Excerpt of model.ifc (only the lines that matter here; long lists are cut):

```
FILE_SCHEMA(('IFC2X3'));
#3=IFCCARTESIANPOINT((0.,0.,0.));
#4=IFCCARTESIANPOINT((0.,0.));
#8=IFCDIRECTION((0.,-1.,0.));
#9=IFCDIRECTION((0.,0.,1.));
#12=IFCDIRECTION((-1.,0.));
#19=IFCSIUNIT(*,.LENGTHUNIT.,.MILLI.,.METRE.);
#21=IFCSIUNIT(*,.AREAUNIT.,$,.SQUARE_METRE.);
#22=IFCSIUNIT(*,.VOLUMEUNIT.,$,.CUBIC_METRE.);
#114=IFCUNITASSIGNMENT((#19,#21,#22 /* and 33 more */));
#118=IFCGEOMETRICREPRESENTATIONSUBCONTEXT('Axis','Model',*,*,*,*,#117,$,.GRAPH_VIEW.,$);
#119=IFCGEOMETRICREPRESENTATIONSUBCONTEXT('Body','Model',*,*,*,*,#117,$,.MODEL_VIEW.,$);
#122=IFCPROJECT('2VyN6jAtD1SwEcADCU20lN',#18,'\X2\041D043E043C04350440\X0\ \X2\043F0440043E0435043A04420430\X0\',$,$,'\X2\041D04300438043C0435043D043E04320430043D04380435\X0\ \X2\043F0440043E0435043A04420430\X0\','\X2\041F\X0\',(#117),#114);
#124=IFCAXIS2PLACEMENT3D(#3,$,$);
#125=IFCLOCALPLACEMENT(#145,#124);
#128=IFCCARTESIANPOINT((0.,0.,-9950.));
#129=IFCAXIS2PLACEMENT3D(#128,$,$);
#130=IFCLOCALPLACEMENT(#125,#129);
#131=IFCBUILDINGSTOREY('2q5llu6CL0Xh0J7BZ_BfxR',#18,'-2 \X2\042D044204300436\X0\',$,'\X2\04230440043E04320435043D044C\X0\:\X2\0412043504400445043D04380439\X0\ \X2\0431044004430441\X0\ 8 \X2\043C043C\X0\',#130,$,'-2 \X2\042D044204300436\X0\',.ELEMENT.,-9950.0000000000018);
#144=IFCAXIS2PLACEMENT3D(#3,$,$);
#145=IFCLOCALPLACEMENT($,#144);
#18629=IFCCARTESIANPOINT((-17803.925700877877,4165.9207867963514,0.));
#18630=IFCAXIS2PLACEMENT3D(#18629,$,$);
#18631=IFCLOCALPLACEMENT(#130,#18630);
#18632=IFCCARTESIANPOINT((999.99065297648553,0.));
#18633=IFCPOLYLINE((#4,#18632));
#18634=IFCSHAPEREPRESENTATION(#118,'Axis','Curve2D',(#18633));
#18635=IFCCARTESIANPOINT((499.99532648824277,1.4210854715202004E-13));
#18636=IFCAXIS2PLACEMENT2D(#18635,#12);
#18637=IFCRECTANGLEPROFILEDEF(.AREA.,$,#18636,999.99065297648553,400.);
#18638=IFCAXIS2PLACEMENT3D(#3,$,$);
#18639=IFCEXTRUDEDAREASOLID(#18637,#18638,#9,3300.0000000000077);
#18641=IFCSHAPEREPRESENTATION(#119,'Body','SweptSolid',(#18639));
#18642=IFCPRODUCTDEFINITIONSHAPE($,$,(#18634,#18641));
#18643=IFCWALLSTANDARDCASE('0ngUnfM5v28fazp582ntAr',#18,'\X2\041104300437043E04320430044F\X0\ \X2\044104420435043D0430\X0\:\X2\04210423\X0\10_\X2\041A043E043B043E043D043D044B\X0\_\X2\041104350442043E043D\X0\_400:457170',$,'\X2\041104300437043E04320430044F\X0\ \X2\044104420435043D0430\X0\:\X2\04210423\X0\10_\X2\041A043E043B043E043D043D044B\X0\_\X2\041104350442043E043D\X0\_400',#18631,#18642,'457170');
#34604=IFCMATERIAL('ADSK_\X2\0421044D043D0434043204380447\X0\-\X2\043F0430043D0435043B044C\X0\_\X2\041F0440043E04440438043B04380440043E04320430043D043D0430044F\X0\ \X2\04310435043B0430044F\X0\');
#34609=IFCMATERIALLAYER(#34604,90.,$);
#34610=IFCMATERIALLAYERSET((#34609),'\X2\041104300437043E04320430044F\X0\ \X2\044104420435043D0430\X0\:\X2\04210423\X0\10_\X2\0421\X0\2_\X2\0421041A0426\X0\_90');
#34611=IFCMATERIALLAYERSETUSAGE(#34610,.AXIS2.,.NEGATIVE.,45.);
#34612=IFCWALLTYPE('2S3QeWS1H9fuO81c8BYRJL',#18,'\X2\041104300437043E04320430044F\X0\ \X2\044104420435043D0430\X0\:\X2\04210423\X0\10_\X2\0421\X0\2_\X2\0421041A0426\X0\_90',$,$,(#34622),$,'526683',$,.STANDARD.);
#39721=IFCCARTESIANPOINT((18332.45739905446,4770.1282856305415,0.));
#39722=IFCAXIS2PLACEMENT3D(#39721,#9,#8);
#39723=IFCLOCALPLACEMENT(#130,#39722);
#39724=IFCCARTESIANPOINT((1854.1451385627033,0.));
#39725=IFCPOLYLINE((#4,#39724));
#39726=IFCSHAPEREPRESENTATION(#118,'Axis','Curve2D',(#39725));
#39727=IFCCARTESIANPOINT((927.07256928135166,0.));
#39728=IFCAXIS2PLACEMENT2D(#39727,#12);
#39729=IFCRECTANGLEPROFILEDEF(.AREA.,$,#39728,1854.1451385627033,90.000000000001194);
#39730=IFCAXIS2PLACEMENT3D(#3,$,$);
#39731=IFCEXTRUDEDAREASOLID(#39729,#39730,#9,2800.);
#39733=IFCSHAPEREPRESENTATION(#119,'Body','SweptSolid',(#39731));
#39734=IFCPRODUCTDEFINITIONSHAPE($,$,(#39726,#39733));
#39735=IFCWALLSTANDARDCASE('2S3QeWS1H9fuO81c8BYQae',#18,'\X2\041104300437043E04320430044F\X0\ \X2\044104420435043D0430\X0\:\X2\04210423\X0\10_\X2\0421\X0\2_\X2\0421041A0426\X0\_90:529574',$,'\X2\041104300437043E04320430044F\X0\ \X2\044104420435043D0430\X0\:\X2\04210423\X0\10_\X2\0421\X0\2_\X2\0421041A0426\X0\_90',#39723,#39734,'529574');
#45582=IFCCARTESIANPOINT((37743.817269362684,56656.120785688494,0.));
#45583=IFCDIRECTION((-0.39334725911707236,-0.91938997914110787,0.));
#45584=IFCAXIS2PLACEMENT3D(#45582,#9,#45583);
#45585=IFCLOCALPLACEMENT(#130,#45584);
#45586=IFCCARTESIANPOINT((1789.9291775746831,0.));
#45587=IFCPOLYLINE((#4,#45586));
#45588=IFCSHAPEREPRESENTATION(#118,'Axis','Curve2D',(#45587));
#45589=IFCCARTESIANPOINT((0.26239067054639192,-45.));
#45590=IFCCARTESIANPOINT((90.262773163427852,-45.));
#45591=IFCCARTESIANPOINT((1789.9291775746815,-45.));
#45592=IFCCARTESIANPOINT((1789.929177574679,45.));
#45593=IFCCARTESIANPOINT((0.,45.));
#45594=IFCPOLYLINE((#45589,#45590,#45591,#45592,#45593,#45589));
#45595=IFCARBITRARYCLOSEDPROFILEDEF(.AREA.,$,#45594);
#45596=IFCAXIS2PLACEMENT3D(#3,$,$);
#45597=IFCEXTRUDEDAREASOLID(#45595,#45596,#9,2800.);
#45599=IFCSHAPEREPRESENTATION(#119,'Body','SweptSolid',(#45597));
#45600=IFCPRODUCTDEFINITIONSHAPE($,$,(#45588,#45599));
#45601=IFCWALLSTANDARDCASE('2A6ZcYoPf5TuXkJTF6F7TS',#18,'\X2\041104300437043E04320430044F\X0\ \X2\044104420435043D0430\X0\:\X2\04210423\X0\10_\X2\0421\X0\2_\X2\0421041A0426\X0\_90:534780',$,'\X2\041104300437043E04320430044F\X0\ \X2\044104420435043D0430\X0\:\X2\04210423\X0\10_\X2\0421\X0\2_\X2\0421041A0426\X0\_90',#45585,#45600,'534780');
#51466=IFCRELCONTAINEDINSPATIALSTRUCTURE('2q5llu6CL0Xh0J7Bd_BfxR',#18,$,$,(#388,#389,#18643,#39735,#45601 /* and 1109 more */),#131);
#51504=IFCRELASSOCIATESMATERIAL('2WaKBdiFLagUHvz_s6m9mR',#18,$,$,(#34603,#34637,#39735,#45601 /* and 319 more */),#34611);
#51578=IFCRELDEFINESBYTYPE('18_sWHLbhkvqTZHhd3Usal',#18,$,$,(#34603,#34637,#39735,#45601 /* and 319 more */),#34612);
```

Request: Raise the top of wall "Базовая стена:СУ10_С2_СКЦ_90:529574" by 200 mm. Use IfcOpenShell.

```python
import ifcopenshell
import ifcopenshell.geom
import ifcopenshell.util.representation
import ifcopenshell.util.shape

model = ifcopenshell.open("model.ifc")
settings = ifcopenshell.geom.settings()


def volume(element):
    """Net volume in cubic metres, openings subtracted."""
    shape = ifcopenshell.geom.create_shape(settings, element)
    return ifcopenshell.util.shape.get_volume(shape.geometry)


wall = model.by_guid("2S3QeWS1H9fuO81c8BYQae")
before = volume(wall)

body = ifcopenshell.util.representation.get_representation(wall, "Model", "Body")
solid = body.Items[0]
old_height = solid.Depth
solid.Depth += 200.0
after = volume(wall)

print(f"height {old_height:g} -> {solid.Depth:g}, volume {before:.3f} -> {after:.3f} m3")

model.write("model-out.ifc")
```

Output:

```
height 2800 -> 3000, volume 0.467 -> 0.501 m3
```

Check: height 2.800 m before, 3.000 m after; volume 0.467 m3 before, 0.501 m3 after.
